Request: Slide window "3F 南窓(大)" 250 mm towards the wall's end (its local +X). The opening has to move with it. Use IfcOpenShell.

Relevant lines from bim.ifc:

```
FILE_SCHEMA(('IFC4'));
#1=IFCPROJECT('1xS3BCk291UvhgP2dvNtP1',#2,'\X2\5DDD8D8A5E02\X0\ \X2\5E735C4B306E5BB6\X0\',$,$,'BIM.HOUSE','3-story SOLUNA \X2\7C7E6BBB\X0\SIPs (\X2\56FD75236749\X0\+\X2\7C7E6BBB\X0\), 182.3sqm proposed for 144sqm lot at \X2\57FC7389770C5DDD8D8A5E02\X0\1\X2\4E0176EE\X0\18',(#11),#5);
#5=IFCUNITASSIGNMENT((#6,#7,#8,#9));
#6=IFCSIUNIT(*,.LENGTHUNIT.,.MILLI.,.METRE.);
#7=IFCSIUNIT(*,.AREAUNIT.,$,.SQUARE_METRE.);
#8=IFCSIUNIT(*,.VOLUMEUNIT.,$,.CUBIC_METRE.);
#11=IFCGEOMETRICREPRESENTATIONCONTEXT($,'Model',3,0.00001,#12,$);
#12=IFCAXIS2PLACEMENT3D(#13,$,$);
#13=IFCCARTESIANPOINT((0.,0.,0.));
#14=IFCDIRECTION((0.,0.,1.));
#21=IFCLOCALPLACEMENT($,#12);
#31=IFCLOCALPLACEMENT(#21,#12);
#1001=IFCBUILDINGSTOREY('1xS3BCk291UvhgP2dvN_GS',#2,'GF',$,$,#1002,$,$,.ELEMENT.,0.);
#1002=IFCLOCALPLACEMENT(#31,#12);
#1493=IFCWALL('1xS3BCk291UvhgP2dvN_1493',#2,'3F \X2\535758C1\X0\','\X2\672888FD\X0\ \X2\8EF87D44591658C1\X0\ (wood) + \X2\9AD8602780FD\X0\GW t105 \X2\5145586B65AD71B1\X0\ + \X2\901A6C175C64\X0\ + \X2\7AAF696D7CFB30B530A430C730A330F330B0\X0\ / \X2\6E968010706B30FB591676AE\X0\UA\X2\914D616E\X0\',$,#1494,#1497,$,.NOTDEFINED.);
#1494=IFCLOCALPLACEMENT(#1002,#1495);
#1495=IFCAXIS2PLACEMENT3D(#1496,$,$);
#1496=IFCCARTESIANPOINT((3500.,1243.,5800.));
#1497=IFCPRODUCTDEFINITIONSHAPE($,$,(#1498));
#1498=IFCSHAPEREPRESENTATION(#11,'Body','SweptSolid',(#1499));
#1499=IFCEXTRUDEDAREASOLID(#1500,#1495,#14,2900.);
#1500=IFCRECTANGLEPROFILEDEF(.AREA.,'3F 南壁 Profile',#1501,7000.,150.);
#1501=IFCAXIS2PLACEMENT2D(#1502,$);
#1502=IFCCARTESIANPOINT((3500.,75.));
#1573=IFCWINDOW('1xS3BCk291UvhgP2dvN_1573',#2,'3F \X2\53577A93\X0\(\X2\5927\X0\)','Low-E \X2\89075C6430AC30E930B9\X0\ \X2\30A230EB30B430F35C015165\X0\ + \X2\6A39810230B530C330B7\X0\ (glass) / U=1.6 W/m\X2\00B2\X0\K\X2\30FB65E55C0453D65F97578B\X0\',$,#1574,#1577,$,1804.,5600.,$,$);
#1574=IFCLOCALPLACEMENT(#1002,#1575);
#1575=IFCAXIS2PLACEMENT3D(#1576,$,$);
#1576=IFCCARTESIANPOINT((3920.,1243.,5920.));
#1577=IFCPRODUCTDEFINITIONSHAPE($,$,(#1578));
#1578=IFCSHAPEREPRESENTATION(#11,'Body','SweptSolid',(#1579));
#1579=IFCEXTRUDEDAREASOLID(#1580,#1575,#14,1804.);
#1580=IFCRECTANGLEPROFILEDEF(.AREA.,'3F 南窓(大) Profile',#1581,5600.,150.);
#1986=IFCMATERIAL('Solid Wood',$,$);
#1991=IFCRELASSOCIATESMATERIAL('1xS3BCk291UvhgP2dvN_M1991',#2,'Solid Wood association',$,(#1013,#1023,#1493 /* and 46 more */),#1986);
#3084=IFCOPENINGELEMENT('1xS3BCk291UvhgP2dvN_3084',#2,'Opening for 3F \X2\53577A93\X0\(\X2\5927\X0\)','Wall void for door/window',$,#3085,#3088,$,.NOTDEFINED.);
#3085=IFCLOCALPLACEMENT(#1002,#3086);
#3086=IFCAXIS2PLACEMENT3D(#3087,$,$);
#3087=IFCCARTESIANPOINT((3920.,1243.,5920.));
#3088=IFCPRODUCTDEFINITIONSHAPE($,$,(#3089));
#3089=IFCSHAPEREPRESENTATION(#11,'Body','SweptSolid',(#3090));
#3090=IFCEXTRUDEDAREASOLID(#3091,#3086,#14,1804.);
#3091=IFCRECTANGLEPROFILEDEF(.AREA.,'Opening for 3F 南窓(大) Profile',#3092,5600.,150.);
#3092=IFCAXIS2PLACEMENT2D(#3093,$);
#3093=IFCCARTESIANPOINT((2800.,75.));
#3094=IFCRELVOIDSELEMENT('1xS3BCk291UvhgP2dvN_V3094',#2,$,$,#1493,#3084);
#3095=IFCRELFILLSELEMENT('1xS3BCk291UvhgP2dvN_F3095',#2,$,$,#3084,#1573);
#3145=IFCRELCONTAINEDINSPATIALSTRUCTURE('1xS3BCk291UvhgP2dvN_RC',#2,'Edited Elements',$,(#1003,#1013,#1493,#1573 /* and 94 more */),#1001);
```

```python
import ifcopenshell
import ifcopenshell.api.geometry
import ifcopenshell.util.placement
import ifcopenshell.util.unit

model = ifcopenshell.open("bim.ifc")
unit_scale = ifcopenshell.util.unit.calculate_unit_scale(model)

window = model.by_guid("1xS3BCk291UvhgP2dvN_1573")
opening = window.FillsVoids[0].RelatingOpeningElement
wall = opening.VoidsElements[0].RelatingBuildingElement

wall_matrix = ifcopenshell.util.placement.get_local_placement(wall.ObjectPlacement)
shift = wall_matrix[:3, 0] * 0.25 / unit_scale
before = ifcopenshell.util.placement.get_local_placement(window.ObjectPlacement)[:3, 3].copy()

# The window is not placed relative to its opening, so move both.
for product in (opening, window):
    matrix = ifcopenshell.util.placement.get_local_placement(product.ObjectPlacement)
    matrix[:3, 3] += shift
    ifcopenshell.api.geometry.edit_object_placement(model, product=product, matrix=matrix, is_si=False)

after = ifcopenshell.util.placement.get_local_placement(window.ObjectPlacement)[:3, 3]
print("window moved by", (after - before).round(3) + 0.0)

model.write("bim_edited.ifc")
```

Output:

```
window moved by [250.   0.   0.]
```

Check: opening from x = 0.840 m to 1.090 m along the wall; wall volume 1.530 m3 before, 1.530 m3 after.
